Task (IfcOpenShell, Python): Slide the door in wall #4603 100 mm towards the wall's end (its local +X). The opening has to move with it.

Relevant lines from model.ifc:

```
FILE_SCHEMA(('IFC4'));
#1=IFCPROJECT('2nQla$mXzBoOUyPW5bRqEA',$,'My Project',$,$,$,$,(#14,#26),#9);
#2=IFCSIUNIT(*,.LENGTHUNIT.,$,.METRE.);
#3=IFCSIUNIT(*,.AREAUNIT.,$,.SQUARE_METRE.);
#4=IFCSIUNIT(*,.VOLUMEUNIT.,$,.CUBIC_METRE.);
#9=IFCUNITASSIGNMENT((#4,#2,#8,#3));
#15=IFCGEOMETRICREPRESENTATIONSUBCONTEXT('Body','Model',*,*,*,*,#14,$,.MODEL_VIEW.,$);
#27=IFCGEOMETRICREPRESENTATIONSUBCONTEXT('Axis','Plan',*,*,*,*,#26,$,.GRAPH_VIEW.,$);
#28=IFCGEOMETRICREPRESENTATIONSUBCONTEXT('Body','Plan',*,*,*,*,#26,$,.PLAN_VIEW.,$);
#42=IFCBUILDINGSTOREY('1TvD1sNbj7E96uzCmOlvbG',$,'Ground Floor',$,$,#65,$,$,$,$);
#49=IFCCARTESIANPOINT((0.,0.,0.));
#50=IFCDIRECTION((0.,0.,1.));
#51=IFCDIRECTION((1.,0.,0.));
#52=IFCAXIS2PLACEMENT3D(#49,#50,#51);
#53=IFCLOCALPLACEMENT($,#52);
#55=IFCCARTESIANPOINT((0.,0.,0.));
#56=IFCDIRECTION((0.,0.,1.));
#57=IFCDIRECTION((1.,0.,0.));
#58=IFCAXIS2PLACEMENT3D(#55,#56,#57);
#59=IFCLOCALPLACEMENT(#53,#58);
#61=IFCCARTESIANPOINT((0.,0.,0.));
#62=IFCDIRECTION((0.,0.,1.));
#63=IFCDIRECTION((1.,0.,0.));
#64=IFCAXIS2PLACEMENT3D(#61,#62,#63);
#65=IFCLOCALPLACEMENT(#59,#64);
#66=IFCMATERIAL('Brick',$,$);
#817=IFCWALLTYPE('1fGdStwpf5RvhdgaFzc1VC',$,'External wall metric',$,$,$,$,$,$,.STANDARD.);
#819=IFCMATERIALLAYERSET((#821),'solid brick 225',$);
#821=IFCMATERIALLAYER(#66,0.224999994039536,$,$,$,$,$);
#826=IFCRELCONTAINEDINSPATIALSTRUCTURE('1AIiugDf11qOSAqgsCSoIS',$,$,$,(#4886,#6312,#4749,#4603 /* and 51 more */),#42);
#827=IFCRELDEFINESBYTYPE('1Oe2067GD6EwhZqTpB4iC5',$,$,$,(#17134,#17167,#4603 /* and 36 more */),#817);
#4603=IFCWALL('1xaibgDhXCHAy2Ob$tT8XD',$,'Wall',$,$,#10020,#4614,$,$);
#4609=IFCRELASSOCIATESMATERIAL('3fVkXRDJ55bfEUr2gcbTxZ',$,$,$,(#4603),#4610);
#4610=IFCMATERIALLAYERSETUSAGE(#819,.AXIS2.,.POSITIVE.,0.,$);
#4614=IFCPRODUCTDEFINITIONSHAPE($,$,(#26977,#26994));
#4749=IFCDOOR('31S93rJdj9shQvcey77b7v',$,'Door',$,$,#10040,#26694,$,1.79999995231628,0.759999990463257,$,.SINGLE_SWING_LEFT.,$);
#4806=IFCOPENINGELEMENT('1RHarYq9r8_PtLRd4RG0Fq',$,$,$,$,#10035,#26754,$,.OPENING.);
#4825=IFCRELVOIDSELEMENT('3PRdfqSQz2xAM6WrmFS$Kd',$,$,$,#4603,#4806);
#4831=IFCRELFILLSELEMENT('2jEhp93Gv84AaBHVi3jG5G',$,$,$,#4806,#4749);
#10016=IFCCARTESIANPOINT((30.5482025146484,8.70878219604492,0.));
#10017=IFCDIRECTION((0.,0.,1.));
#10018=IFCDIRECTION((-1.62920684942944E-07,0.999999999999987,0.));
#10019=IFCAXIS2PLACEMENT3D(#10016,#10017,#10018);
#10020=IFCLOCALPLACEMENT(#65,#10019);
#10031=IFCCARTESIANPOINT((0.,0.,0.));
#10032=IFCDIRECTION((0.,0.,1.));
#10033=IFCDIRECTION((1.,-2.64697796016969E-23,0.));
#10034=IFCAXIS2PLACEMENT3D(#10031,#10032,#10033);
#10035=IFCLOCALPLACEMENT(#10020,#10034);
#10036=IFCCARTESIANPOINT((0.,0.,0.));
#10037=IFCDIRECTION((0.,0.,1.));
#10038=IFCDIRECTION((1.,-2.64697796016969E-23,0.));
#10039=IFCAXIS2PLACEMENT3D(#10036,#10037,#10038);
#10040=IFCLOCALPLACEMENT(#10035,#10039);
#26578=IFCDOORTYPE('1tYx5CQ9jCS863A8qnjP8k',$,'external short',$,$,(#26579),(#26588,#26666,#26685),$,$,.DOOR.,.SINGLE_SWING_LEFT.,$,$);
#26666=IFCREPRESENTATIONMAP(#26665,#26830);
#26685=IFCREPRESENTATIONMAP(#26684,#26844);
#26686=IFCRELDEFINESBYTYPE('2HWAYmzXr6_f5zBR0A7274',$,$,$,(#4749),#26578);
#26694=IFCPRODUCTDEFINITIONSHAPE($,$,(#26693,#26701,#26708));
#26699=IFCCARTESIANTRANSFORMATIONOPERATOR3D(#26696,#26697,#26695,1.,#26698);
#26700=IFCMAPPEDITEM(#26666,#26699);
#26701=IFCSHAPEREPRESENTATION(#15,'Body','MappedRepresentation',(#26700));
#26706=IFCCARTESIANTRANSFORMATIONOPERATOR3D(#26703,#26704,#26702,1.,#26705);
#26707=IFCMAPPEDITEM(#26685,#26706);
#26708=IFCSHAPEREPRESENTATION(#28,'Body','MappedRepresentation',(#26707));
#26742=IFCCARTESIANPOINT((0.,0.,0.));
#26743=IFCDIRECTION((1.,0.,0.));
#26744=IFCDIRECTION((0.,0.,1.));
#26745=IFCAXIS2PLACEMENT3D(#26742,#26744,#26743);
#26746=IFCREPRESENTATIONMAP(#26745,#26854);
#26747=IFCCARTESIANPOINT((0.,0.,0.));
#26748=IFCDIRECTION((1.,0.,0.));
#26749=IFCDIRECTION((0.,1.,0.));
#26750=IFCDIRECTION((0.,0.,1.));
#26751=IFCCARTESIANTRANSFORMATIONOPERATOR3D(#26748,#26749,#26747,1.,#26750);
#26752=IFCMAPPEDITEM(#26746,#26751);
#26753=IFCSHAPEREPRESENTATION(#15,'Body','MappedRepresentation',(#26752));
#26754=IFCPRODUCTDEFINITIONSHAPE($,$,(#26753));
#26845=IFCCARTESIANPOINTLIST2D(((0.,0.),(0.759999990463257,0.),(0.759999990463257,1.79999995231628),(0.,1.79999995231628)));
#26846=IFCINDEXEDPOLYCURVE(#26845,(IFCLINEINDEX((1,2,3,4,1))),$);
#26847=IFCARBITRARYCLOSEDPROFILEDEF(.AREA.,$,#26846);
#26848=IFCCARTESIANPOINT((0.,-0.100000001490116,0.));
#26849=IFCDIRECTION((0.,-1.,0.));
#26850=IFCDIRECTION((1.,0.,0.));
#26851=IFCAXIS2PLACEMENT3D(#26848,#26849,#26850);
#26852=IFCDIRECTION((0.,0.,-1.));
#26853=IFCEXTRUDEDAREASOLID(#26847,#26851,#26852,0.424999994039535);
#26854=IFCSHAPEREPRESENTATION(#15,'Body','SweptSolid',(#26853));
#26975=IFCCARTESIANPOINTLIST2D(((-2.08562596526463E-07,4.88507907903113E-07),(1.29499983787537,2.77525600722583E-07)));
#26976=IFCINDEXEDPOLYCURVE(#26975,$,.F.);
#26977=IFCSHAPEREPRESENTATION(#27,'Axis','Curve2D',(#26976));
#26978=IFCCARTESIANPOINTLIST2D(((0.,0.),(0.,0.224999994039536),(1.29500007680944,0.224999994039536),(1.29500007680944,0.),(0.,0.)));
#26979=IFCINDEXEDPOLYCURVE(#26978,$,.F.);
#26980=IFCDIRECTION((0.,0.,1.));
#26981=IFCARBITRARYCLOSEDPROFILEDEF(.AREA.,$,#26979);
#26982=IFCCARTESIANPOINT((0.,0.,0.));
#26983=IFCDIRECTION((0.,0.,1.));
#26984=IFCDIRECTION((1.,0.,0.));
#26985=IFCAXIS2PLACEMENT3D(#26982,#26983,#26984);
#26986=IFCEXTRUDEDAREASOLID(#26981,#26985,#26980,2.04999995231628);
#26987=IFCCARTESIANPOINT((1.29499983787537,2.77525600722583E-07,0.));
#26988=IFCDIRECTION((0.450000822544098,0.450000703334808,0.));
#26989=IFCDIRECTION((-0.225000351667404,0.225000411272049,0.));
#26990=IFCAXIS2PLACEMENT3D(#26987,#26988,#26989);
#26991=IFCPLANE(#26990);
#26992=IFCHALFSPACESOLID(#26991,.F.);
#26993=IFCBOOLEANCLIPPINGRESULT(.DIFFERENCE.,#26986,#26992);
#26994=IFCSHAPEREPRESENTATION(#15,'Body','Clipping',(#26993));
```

```python
import ifcopenshell
import ifcopenshell.api.geometry
import ifcopenshell.util.placement
import ifcopenshell.util.unit

model = ifcopenshell.open("model.ifc")
unit_scale = ifcopenshell.util.unit.calculate_unit_scale(model)

door = model.by_guid("31S93rJdj9shQvcey77b7v")
opening = door.FillsVoids[0].RelatingOpeningElement
wall = opening.VoidsElements[0].RelatingBuildingElement

wall_matrix = ifcopenshell.util.placement.get_local_placement(wall.ObjectPlacement)
shift = wall_matrix[:3, 0] * 0.1 / unit_scale
before = ifcopenshell.util.placement.get_local_placement(door.ObjectPlacement)[:3, 3].copy()

# The door is placed relative to its opening, so it follows when the opening moves.
matrix = ifcopenshell.util.placement.get_local_placement(opening.ObjectPlacement)
matrix[:3, 3] += shift
ifcopenshell.api.geometry.edit_object_placement(
    model, product=opening, matrix=matrix, is_si=False, should_transform_children=True
)

after = ifcopenshell.util.placement.get_local_placement(door.ObjectPlacement)[:3, 3]
print("door moved by", (after - before).round(3) + 0.0)

model.write("model_edited.ifc")
```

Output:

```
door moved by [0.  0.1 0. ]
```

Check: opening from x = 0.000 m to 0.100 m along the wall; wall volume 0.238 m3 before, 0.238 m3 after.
